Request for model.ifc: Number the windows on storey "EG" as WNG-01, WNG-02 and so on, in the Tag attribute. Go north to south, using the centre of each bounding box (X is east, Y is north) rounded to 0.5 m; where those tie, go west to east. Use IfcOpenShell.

First a look at what the model holds.

```python
import ifcopenshell
import ifcopenshell.util.element
import ifcopenshell.util.placement

model = ifcopenshell.open("model.ifc")
print(model.schema)
storey = next(s for s in model.by_type("IfcBuildingStorey") if s.Name == "EG")
windows = [e for e in ifcopenshell.util.element.get_decomposition(storey) if e.is_a("IfcWindow")]
for e in sorted(windows, key=lambda e: e.id()):
    origin = ifcopenshell.util.placement.get_local_placement(e.ObjectPlacement)[:3, 3]
    print(e.id(), e.Tag, e.Name, origin.round(2) + 0.0, sep=" | ")
```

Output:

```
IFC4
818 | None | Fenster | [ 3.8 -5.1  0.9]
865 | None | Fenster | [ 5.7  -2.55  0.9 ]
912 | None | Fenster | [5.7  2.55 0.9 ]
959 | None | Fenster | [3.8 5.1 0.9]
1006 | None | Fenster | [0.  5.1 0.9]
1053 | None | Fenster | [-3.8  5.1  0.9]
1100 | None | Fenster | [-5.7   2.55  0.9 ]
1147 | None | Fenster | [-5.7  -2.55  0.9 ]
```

```python
import ifcopenshell
import ifcopenshell.geom
import ifcopenshell.util.element
import ifcopenshell.util.shape

model = ifcopenshell.open("model.ifc")
settings = ifcopenshell.geom.settings()
settings.set("use-world-coords", True)


def centre(element):
    shape = ifcopenshell.geom.create_shape(settings, element)
    return ifcopenshell.util.shape.get_bbox_centroid(shape.geometry)


storey = next(s for s in model.by_type("IfcBuildingStorey") if s.Name == "EG")
windows = [e for e in ifcopenshell.util.element.get_decomposition(storey) if e.is_a("IfcWindow")]

# Insertion points can sit at a corner or the storey origin, so sort by the geometry (in metres).
centres = {e: centre(e) for e in windows}
windows.sort(key=lambda e: (-round(centres[e][1] / 0.5), centres[e][0]))

for i, e in enumerate(windows, start=1):
    number = f"WNG-{i:02d}"
    e.Tag = number
    print(e.id(), number)

model.write("model_edited.ifc")
```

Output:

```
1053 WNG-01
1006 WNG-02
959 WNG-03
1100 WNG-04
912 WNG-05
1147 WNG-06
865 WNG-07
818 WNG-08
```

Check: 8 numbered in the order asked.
